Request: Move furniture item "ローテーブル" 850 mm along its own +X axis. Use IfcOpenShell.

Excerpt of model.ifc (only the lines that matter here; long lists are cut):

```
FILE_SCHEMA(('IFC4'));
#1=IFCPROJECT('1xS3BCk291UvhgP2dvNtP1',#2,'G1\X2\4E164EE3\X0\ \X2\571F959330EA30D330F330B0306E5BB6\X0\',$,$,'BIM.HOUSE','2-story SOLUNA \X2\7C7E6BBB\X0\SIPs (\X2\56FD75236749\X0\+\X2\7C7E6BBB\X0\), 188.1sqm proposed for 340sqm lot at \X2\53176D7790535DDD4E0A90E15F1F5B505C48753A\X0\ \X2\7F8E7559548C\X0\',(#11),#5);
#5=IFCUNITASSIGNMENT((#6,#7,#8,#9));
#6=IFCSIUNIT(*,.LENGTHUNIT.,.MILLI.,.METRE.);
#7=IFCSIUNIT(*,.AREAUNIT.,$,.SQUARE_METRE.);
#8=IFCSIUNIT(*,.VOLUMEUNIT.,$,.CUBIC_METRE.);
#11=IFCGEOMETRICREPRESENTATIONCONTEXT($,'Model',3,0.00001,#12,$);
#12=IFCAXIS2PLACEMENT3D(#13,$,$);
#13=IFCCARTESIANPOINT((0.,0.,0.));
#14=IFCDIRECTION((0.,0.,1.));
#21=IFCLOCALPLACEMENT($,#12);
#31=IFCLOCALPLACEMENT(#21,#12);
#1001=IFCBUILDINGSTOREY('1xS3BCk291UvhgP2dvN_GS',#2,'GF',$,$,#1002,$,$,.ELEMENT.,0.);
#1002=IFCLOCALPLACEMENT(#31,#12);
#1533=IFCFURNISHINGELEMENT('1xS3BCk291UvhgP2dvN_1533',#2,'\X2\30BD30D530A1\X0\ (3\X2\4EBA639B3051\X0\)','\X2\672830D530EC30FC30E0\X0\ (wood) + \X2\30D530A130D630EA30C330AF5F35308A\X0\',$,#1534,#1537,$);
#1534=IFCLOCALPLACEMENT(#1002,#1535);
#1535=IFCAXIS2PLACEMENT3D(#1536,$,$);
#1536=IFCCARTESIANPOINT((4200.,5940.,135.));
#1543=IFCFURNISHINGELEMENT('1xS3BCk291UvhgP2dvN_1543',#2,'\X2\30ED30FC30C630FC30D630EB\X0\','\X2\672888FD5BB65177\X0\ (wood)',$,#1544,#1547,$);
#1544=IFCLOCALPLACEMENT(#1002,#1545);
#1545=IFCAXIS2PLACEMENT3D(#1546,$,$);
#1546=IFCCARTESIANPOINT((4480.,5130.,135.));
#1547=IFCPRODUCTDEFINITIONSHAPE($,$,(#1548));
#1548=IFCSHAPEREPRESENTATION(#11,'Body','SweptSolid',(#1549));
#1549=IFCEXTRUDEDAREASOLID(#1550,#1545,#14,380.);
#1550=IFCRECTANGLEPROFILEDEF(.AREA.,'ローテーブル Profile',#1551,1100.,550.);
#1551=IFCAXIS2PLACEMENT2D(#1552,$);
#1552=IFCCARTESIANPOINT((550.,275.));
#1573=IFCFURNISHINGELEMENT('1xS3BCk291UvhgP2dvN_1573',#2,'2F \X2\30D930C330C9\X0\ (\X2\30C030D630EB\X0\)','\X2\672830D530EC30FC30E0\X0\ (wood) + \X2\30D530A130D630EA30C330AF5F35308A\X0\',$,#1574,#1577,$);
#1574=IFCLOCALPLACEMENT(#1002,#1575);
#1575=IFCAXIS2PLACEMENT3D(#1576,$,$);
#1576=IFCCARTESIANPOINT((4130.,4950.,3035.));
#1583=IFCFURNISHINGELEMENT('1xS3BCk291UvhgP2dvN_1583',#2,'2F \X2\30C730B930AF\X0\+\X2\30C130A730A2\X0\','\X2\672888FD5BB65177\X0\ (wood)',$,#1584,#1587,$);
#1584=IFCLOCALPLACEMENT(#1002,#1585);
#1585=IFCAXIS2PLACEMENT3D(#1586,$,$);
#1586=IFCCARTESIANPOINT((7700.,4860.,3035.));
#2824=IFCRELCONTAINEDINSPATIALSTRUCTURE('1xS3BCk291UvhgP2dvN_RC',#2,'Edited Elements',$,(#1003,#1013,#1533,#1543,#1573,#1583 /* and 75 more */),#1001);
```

```python
import ifcopenshell
import ifcopenshell.api.geometry
import ifcopenshell.util.placement
import ifcopenshell.util.unit

model = ifcopenshell.open("model.ifc")
unit_scale = ifcopenshell.util.unit.calculate_unit_scale(model)

item = model.by_guid("1xS3BCk291UvhgP2dvN_1543")
matrix = ifcopenshell.util.placement.get_local_placement(item.ObjectPlacement)
matrix[:3, 3] += matrix[:3, 0] * 0.85 / unit_scale
ifcopenshell.api.geometry.edit_object_placement(model, product=item, matrix=matrix, is_si=False)

print(ifcopenshell.util.placement.get_local_placement(item.ObjectPlacement).round(3) + 0.0)

model.write("model_updated.ifc")
```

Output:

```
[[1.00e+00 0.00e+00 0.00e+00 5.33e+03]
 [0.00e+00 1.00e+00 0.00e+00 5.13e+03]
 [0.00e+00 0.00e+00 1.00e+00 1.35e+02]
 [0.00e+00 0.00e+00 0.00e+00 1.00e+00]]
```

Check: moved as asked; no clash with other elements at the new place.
